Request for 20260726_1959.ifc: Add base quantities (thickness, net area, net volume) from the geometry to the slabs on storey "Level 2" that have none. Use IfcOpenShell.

First a look at what the model holds.

```python
import ifcopenshell
import ifcopenshell.util.element
import ifcopenshell.util.unit

model = ifcopenshell.open("20260726_1959.ifc")
print(model.schema)
for unit_type in ("LENGTHUNIT", "AREAUNIT", "VOLUMEUNIT"):
    print(unit_type, ifcopenshell.util.unit.calculate_unit_scale(model, unit_type))
storey = next(s for s in model.by_type("IfcBuildingStorey") if s.Name == "Level 2")
slabs = [e for e in ifcopenshell.util.element.get_decomposition(storey) if e.is_a("IfcSlab")]
for e in sorted(slabs, key=lambda e: e.id()):
    print(e.id(), e.is_a(), e.Name, list(ifcopenshell.util.element.get_psets(e, qtos_only=True)), sep=" | ")
```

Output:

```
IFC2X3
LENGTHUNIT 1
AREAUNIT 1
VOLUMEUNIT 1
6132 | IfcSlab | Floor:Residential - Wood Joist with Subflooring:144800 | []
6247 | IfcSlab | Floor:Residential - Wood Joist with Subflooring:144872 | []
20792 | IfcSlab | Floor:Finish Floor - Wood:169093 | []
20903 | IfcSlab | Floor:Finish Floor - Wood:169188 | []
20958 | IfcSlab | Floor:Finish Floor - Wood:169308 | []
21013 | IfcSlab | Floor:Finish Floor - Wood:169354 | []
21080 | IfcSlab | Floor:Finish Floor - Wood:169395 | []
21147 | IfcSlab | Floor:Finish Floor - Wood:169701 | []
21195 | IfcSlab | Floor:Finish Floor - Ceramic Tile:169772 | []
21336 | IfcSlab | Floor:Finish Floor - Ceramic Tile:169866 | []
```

```python
import ifcopenshell
import ifcopenshell.api.pset
import ifcopenshell.geom
import ifcopenshell.util.element
import ifcopenshell.util.shape
import ifcopenshell.util.unit

model = ifcopenshell.open("20260726_1959.ifc")
unit_scale = ifcopenshell.util.unit.calculate_unit_scale(model)
area_scale = ifcopenshell.util.unit.calculate_unit_scale(model, "AREAUNIT")
volume_scale = ifcopenshell.util.unit.calculate_unit_scale(model, "VOLUMEUNIT")
settings = ifcopenshell.geom.settings()

storey = next(s for s in model.by_type("IfcBuildingStorey") if s.Name == "Level 2")
slabs = [e for e in ifcopenshell.util.element.get_decomposition(storey) if e.is_a("IfcSlab")]

for e in sorted(slabs, key=lambda e: e.id()):
    if ifcopenshell.util.element.get_psets(e, qtos_only=True, should_inherit=False):
        continue
    # Geometry comes back in metres, in the element's own axes.
    shape = ifcopenshell.geom.create_shape(settings, e)
    values = {
        "Width": ifcopenshell.util.shape.get_z(shape.geometry) / unit_scale,
        "NetArea": ifcopenshell.util.shape.get_footprint_area(shape.geometry) / area_scale,
        "NetVolume": ifcopenshell.util.shape.get_volume(shape.geometry) / volume_scale,
    }
    qto = ifcopenshell.api.pset.add_qto(model, product=e, name="BaseQuantities")
    ifcopenshell.api.pset.edit_qto(model, qto=qto, properties=values)
    print(e.id(), {k: round(v, 3) for k, v in values.items()})

model.write("20260726_1959_edited.ifc")
```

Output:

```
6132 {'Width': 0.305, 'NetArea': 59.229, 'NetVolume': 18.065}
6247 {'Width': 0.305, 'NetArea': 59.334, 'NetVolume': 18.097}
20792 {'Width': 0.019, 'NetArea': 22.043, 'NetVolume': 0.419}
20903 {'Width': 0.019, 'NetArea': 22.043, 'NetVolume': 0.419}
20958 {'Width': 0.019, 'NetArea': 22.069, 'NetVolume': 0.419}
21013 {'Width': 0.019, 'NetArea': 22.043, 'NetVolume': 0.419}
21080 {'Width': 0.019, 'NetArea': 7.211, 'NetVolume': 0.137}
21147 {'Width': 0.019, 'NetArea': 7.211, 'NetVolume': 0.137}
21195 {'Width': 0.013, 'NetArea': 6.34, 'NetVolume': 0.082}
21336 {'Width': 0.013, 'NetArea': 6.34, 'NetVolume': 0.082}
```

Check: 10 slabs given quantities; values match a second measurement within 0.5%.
